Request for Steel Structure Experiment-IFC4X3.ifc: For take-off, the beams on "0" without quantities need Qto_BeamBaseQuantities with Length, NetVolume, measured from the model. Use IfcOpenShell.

First a look at what the model holds.

```python
import ifcopenshell
import ifcopenshell.util.element
import ifcopenshell.util.unit

model = ifcopenshell.open("Steel Structure Experiment-IFC4X3.ifc")
print(model.schema)
for unit_type in ("LENGTHUNIT", "AREAUNIT", "VOLUMEUNIT"):
    print(unit_type, ifcopenshell.util.unit.calculate_unit_scale(model, unit_type))
storey = next(s for s in model.by_type("IfcBuildingStorey") if s.Name == "0")
beams = [e for e in ifcopenshell.util.element.get_decomposition(storey) if e.is_a("IfcBeam")]
for e in sorted(beams, key=lambda e: e.id()):
    print(e.id(), e.is_a(), e.Name, list(ifcopenshell.util.element.get_psets(e, qtos_only=True)), sep=" | ")
```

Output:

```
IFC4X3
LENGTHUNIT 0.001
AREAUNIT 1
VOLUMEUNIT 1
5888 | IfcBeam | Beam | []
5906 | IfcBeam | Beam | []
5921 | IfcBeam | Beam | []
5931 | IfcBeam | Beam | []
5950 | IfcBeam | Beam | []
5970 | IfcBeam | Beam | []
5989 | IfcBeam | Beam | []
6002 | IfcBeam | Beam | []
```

```python
import ifcopenshell
import ifcopenshell.api.pset
import ifcopenshell.geom
import ifcopenshell.util.element
import ifcopenshell.util.shape
import ifcopenshell.util.unit

model = ifcopenshell.open("Steel Structure Experiment-IFC4X3.ifc")
unit_scale = ifcopenshell.util.unit.calculate_unit_scale(model)
volume_scale = ifcopenshell.util.unit.calculate_unit_scale(model, "VOLUMEUNIT")
settings = ifcopenshell.geom.settings()

storey = next(s for s in model.by_type("IfcBuildingStorey") if s.Name == "0")
beams = [e for e in ifcopenshell.util.element.get_decomposition(storey) if e.is_a("IfcBeam")]

for e in sorted(beams, key=lambda e: e.id()):
    if ifcopenshell.util.element.get_psets(e, qtos_only=True, should_inherit=False):
        continue
    # Geometry comes back in metres, in the element's own axes.
    shape = ifcopenshell.geom.create_shape(settings, e)
    values = {
        "Length": ifcopenshell.util.shape.get_max_xyz(shape.geometry) / unit_scale,
        "NetVolume": ifcopenshell.util.shape.get_volume(shape.geometry) / volume_scale,
    }
    qto = ifcopenshell.api.pset.add_qto(model, product=e, name="Qto_BeamBaseQuantities")
    ifcopenshell.api.pset.edit_qto(model, qto=qto, properties=values)
    print(e.id(), {k: round(v, 3) for k, v in values.items()})

model.write("Steel Structure Experiment-IFC4X3_edited.ifc")
```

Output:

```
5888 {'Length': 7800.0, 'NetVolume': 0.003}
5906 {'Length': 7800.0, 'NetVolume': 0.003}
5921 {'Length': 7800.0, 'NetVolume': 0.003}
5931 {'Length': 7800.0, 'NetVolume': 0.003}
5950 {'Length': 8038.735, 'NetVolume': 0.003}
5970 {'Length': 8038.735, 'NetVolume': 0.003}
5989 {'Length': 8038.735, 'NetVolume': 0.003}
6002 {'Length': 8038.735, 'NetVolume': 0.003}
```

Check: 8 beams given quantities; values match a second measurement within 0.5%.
